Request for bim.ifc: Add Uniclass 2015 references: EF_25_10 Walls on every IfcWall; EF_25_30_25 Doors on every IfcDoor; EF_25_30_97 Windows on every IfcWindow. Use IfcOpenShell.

First a look at what the model holds.

```python
import ifcopenshell

model = ifcopenshell.open("bim.ifc")
print(model.schema)
print("classifications:", [c.Name for c in model.by_type("IfcClassification")])
for ifc_class in ("IfcDoor", "IfcRoof", "IfcStair", "IfcWall", "IfcWindow"):
    print(ifc_class, len(model.by_type(ifc_class)))
```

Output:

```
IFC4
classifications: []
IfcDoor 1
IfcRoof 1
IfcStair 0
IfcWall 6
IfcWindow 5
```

```python
import ifcopenshell
import ifcopenshell.api.classification

model = ifcopenshell.open("bim.ifc")

system = ifcopenshell.api.classification.add_classification(model, classification="Uniclass 2015")

codes = {
    "IfcWall": ("EF_25_10", "Walls"),
    "IfcDoor": ("EF_25_30_25", "Doors"),
    "IfcWindow": ("EF_25_30_97", "Windows"),
}
for ifc_class, (code, name) in codes.items():
    products = model.by_type(ifc_class)
    ifcopenshell.api.classification.add_reference(
        model, products=products, classification=system, identification=code, name=name
    )
    print(code, len(products))

model.write("bim_v2.ifc")
```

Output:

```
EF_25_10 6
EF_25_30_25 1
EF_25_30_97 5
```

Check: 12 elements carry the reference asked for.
